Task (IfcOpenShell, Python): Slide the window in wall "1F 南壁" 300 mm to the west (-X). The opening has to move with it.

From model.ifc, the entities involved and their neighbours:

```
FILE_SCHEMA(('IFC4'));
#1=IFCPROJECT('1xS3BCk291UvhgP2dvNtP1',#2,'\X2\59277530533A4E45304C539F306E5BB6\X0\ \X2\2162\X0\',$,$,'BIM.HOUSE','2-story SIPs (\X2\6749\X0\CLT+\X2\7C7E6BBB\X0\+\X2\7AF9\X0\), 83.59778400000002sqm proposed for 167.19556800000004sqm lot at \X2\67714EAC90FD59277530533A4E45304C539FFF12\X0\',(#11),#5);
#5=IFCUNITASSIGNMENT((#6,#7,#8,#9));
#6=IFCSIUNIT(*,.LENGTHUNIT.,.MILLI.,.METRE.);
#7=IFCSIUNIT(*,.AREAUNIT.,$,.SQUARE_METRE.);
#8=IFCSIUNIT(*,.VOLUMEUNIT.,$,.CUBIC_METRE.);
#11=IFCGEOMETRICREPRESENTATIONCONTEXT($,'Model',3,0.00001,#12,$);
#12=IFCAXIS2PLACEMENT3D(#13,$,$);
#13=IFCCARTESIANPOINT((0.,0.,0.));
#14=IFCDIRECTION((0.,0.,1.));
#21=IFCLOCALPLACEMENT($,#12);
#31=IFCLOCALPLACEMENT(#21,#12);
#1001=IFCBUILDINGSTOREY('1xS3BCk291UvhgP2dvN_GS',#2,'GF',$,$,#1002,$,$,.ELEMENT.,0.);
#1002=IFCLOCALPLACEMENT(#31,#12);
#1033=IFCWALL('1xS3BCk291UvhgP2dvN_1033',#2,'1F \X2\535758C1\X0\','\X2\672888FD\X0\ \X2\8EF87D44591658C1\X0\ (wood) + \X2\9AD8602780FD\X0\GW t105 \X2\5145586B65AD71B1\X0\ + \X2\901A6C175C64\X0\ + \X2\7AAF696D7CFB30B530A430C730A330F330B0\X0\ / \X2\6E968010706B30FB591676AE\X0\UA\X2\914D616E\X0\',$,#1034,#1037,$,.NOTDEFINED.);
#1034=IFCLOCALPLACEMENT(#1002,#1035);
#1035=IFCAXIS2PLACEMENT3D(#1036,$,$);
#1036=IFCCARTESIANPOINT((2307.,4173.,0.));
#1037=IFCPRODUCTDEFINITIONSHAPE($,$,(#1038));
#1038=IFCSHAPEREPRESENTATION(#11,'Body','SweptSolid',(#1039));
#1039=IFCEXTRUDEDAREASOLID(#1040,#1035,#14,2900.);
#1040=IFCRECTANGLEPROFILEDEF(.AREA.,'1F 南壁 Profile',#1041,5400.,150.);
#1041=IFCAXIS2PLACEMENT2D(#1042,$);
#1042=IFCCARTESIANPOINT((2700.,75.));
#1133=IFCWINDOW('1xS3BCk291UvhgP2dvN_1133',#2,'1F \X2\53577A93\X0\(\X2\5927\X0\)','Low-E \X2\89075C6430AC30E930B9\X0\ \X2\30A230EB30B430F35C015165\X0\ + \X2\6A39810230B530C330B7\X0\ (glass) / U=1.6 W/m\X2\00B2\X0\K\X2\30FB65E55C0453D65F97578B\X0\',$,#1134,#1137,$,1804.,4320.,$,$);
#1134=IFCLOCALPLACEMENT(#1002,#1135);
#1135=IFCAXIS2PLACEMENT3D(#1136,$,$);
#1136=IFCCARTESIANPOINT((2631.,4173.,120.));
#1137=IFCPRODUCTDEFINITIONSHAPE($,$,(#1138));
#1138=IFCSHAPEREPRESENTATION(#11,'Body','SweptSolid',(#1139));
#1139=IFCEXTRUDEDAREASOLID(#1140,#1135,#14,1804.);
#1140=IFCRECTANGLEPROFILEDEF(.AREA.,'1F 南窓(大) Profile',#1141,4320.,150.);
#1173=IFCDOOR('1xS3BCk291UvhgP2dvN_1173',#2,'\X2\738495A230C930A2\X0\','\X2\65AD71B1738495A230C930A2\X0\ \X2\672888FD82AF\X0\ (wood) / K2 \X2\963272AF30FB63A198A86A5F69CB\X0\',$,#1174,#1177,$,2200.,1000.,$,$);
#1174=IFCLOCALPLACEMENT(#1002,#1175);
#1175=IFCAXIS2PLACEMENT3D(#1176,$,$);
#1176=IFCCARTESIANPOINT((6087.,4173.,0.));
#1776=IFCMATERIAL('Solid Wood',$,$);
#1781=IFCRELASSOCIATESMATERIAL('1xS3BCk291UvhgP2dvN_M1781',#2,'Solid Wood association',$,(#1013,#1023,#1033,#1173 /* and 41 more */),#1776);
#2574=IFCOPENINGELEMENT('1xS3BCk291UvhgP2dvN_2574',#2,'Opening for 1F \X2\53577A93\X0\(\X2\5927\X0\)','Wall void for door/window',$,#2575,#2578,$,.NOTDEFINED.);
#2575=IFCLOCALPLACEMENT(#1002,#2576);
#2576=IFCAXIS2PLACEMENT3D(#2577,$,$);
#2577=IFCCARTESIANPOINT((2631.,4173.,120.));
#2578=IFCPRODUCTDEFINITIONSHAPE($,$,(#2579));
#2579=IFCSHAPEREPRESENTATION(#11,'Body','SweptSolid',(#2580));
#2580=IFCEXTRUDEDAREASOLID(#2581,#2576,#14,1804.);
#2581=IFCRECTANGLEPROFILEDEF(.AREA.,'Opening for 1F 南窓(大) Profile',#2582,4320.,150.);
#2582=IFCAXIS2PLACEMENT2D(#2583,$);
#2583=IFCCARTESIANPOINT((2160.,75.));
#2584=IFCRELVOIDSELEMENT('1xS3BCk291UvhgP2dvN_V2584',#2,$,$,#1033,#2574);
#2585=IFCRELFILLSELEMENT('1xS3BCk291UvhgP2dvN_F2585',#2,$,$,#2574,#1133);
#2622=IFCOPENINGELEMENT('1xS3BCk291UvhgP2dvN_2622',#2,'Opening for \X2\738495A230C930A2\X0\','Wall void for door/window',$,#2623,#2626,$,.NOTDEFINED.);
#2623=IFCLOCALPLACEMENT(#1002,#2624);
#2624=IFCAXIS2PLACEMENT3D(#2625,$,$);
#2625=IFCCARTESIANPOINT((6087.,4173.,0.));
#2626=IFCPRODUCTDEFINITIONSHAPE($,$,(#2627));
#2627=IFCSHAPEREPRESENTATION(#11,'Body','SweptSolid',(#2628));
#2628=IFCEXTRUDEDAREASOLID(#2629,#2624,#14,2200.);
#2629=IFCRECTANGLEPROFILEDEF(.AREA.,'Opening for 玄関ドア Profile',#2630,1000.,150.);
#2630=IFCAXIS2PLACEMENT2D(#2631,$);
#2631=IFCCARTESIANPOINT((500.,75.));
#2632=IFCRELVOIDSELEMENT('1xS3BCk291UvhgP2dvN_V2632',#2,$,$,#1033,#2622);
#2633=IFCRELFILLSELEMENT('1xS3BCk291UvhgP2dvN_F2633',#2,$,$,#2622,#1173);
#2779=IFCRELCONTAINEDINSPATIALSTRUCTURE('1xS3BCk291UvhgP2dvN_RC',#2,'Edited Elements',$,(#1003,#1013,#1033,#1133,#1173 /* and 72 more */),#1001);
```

```python
import ifcopenshell
import ifcopenshell.api.geometry
import ifcopenshell.util.placement

model = ifcopenshell.open("model.ifc")

window = model.by_guid("1xS3BCk291UvhgP2dvN_1133")
opening = window.FillsVoids[0].RelatingOpeningElement
wall = opening.VoidsElements[0].RelatingBuildingElement

wall_matrix = ifcopenshell.util.placement.get_local_placement(wall.ObjectPlacement)
shift = wall_matrix[:3, 0] * -300.0
before = ifcopenshell.util.placement.get_local_placement(window.ObjectPlacement)[:3, 3].copy()

# The window is not placed relative to its opening, so move both.
for product in (opening, window):
    matrix = ifcopenshell.util.placement.get_local_placement(product.ObjectPlacement)
    matrix[:3, 3] += shift
    ifcopenshell.api.geometry.edit_object_placement(model, product=product, matrix=matrix, is_si=False)

after = ifcopenshell.util.placement.get_local_placement(window.ObjectPlacement)[:3, 3]
print("window moved by", (after - before).round(3) + 0.0)

model.write("model_v2.ifc")
```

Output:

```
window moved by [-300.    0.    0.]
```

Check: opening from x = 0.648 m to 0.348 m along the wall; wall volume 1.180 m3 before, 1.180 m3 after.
